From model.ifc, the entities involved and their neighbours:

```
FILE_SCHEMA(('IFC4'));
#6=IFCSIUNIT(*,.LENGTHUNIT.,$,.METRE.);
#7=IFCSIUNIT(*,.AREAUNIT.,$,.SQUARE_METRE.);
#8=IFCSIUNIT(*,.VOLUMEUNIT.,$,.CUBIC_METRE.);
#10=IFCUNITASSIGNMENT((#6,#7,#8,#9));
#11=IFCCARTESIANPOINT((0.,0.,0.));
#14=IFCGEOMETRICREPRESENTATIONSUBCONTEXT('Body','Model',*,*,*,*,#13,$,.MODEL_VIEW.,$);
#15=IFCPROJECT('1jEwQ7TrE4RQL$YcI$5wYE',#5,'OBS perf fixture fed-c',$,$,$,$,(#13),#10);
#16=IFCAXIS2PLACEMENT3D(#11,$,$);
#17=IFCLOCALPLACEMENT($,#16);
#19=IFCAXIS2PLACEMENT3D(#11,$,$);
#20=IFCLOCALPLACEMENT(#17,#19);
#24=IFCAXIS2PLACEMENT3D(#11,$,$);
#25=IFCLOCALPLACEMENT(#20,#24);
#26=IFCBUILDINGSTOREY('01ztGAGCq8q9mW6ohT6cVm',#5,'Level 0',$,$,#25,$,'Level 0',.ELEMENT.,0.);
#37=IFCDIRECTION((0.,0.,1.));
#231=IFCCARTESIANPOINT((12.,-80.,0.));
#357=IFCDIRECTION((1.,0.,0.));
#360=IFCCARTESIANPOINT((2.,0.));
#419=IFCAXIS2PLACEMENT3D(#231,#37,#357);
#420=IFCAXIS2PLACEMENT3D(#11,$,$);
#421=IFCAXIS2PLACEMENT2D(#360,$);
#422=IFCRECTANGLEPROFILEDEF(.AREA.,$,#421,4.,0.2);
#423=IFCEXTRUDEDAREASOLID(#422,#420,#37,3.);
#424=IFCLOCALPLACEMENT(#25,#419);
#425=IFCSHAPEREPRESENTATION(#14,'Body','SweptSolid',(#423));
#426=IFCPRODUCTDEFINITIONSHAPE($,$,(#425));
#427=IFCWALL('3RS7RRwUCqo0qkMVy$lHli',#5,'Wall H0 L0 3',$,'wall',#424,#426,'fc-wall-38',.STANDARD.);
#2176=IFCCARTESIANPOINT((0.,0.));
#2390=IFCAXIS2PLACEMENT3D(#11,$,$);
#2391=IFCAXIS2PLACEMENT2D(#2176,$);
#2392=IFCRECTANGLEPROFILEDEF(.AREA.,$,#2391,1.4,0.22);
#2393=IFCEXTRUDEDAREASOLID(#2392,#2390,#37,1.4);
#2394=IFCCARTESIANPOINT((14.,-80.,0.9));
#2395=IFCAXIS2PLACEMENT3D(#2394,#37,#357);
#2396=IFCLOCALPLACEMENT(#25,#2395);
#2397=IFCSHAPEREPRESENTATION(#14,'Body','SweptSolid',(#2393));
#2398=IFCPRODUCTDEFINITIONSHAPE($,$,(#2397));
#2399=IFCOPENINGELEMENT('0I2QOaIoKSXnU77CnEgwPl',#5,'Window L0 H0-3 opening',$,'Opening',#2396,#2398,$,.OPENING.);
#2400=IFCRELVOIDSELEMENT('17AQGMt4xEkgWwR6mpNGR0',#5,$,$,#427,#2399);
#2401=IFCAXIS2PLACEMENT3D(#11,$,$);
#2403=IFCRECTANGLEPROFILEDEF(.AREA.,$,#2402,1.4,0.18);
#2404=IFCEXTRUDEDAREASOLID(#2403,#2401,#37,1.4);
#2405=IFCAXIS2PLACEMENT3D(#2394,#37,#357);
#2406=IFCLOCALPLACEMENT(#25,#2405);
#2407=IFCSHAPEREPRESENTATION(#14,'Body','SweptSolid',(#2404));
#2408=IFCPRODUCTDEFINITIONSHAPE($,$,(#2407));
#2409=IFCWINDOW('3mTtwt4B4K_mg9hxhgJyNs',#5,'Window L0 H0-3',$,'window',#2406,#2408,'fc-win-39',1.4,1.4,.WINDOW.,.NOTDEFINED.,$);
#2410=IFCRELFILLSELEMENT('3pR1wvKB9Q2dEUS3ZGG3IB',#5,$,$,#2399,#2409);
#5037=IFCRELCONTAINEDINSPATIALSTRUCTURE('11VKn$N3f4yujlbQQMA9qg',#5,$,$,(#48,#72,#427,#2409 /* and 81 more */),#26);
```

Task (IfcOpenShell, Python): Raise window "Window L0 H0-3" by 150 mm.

```python
import numpy as np
import ifcopenshell
import ifcopenshell.api.geometry
import ifcopenshell.util.placement
import ifcopenshell.util.unit

model = ifcopenshell.open("model.ifc")
unit_scale = ifcopenshell.util.unit.calculate_unit_scale(model)

window = model.by_guid("3mTtwt4B4K_mg9hxhgJyNs")
opening = window.FillsVoids[0].RelatingOpeningElement
dz = 0.15 / unit_scale

shift = np.array([0.0, 0.0, dz])
# The window is not placed relative to its opening, so move both.
for product in (opening, window):
    matrix = ifcopenshell.util.placement.get_local_placement(product.ObjectPlacement)
    matrix[:3, 3] += shift
    ifcopenshell.api.geometry.edit_object_placement(model, product=product, matrix=matrix, is_si=False)

print(f"moved by {dz * unit_scale:+.3f} m")

model.write("model-out.ifc")
```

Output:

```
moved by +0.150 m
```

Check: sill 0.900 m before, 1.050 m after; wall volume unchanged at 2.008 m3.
